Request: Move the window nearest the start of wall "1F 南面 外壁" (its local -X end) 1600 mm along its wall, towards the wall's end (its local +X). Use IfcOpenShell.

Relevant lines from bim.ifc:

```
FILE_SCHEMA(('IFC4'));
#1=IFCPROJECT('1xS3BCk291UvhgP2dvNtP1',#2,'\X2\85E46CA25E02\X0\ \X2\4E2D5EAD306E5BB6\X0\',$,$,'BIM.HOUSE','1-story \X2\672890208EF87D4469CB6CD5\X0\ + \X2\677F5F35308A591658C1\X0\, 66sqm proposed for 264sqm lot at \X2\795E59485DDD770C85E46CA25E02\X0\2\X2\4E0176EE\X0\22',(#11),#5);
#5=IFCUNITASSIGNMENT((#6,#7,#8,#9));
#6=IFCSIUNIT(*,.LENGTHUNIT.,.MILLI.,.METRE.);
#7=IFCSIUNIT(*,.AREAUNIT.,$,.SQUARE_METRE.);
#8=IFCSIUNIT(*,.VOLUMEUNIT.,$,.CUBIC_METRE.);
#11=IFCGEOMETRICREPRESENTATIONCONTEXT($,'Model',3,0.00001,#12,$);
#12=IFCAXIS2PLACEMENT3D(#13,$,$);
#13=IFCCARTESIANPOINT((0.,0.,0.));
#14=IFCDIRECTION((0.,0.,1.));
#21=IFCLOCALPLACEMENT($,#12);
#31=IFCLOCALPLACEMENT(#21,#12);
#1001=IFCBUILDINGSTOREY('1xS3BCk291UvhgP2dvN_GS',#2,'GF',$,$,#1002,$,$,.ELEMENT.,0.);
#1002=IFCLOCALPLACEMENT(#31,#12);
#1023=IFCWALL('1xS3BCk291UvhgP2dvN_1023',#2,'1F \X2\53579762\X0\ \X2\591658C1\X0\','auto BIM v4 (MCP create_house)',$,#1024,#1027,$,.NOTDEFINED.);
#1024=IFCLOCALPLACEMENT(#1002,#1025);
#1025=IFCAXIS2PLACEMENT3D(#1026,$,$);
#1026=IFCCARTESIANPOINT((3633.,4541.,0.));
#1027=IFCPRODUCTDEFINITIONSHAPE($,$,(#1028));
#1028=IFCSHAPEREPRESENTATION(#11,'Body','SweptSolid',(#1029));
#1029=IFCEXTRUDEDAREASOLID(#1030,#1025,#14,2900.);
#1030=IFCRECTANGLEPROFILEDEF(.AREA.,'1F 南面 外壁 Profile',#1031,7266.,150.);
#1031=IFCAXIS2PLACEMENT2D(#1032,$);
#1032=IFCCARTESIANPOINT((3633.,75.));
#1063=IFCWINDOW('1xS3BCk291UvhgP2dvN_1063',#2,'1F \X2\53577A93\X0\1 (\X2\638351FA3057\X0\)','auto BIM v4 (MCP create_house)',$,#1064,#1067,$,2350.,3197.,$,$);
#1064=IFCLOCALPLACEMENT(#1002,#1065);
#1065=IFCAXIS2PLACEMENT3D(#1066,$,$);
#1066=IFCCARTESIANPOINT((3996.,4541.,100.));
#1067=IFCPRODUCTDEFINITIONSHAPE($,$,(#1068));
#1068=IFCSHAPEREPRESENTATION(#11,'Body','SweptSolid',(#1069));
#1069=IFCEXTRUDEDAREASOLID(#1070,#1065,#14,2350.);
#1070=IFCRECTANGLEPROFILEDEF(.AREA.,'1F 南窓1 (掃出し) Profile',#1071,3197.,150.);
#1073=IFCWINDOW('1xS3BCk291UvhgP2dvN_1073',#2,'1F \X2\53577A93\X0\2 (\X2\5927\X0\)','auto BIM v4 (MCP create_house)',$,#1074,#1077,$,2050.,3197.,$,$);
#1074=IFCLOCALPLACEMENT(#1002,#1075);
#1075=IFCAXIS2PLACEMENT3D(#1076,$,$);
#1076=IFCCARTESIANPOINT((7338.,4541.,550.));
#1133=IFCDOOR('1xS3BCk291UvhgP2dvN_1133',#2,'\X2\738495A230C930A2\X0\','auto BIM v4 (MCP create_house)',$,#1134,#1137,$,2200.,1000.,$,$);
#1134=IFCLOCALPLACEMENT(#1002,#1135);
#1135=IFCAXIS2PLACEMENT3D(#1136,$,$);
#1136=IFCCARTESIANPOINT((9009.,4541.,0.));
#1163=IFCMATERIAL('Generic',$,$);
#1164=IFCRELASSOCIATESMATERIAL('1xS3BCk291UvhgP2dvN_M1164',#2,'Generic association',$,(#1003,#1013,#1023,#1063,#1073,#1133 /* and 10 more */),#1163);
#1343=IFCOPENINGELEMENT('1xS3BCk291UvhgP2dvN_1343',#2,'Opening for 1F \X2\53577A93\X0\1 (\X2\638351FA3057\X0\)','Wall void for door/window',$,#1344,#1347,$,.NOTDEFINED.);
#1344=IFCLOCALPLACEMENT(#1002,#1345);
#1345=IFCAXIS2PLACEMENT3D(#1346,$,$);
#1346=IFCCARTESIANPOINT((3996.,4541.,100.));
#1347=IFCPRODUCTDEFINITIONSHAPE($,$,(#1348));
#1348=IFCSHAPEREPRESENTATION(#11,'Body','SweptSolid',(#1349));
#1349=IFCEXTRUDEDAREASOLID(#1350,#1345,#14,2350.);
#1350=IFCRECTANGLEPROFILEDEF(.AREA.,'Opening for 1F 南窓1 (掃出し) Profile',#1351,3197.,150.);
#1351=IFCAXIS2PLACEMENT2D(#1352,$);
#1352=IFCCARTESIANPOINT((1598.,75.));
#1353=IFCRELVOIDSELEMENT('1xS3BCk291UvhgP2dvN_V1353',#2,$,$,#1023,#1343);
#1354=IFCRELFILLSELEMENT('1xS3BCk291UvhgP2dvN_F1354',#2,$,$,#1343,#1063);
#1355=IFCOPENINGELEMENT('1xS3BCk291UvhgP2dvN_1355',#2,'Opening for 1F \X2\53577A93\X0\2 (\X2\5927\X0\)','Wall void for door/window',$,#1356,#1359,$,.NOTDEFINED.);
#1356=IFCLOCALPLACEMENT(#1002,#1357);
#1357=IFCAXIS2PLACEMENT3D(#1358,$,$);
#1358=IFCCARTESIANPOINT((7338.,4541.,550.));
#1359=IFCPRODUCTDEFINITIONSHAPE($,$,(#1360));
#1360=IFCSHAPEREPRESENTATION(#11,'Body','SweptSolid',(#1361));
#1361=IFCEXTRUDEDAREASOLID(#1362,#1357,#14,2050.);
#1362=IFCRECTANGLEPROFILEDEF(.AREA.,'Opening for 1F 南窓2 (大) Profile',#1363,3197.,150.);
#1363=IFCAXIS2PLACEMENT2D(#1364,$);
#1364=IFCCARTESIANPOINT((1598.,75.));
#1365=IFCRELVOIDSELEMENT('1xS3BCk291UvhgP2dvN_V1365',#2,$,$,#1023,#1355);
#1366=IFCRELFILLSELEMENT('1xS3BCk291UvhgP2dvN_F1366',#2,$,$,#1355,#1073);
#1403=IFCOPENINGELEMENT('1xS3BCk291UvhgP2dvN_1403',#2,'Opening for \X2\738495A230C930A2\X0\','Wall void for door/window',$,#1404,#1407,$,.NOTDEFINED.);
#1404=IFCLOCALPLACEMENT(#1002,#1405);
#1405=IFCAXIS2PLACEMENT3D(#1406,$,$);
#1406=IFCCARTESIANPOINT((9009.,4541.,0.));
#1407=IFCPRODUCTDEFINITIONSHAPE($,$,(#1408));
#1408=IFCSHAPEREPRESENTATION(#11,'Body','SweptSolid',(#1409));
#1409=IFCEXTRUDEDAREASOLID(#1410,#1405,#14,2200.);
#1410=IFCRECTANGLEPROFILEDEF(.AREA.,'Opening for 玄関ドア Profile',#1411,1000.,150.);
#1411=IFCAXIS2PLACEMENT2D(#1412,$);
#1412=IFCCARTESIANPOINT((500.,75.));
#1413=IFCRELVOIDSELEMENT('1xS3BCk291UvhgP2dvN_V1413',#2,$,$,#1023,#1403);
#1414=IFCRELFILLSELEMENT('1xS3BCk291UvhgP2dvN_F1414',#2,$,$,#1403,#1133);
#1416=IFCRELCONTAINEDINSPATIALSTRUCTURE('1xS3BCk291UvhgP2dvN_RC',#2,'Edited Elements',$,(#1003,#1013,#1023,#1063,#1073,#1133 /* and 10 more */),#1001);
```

```python
import ifcopenshell
import ifcopenshell.api.geometry
import ifcopenshell.util.placement
import ifcopenshell.util.unit

model = ifcopenshell.open("bim.ifc")
unit_scale = ifcopenshell.util.unit.calculate_unit_scale(model)

window = model.by_guid("1xS3BCk291UvhgP2dvN_1063")
opening = window.FillsVoids[0].RelatingOpeningElement
wall = opening.VoidsElements[0].RelatingBuildingElement

wall_matrix = ifcopenshell.util.placement.get_local_placement(wall.ObjectPlacement)
shift = wall_matrix[:3, 0] * 1.6 / unit_scale
before = ifcopenshell.util.placement.get_local_placement(window.ObjectPlacement)[:3, 3].copy()

# The window is not placed relative to its opening, so move both.
for product in (opening, window):
    matrix = ifcopenshell.util.placement.get_local_placement(product.ObjectPlacement)
    matrix[:3, 3] += shift
    ifcopenshell.api.geometry.edit_object_placement(model, product=product, matrix=matrix, is_si=False)

after = ifcopenshell.util.placement.get_local_placement(window.ObjectPlacement)[:3, 3]
print("window moved by", (after - before).round(3) + 0.0)

model.write("bim-out.ifc")
```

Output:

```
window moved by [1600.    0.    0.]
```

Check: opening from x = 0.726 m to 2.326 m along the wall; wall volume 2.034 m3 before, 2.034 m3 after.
